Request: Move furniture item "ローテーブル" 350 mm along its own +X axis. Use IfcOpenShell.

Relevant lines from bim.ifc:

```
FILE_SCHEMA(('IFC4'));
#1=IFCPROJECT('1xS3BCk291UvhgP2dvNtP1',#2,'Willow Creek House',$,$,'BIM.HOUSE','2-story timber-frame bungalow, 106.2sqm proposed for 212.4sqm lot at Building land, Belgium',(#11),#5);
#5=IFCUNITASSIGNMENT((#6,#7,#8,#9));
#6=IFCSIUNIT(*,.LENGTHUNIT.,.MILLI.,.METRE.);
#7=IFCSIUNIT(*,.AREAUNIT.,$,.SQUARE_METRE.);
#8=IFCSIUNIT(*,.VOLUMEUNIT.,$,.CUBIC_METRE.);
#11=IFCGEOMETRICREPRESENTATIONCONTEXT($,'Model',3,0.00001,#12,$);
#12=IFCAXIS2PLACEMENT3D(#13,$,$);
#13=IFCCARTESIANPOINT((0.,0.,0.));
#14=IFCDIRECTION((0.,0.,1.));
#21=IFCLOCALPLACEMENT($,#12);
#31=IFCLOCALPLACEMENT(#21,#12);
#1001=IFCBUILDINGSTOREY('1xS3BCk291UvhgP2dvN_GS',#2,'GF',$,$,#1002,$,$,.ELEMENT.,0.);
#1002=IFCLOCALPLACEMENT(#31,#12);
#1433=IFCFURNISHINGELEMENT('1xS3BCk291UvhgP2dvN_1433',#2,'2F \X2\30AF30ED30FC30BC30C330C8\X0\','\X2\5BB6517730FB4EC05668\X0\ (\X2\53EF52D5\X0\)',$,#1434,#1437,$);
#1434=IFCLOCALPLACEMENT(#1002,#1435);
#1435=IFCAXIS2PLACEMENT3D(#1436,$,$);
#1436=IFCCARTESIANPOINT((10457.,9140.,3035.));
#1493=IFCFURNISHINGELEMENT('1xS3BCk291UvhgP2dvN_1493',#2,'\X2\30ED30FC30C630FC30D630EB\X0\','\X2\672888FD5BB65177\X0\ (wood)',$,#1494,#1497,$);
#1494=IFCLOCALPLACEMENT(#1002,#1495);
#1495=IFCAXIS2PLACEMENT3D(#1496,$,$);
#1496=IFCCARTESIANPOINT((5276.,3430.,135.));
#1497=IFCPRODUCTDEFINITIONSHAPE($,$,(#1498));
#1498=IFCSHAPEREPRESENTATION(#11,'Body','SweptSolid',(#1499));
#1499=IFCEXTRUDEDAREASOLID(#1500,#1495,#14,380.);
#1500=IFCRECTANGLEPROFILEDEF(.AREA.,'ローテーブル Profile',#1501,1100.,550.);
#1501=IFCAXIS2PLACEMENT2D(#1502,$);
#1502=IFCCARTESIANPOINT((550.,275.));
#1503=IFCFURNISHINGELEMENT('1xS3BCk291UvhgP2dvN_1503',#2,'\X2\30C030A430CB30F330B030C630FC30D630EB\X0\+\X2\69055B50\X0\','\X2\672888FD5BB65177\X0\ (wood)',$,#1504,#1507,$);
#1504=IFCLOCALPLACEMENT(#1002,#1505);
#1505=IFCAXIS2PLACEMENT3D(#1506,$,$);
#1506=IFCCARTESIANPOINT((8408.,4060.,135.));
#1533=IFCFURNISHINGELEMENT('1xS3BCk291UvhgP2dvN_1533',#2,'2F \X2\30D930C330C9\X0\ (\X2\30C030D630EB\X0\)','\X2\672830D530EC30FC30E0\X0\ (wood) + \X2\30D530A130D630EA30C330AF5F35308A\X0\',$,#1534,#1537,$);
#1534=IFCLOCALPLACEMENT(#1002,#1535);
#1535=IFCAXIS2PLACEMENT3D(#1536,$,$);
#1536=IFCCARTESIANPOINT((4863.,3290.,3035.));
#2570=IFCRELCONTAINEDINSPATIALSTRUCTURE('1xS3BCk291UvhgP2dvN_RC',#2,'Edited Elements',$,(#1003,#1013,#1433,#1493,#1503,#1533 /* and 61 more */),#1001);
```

```python
import ifcopenshell
import ifcopenshell.api.geometry
import ifcopenshell.util.placement
import ifcopenshell.util.unit

model = ifcopenshell.open("bim.ifc")
unit_scale = ifcopenshell.util.unit.calculate_unit_scale(model)

item = model.by_id(1493)
matrix = ifcopenshell.util.placement.get_local_placement(item.ObjectPlacement)
matrix[:3, 3] += matrix[:3, 0] * 0.35 / unit_scale
ifcopenshell.api.geometry.edit_object_placement(model, product=item, matrix=matrix, is_si=False)

print(ifcopenshell.util.placement.get_local_placement(item.ObjectPlacement).round(3) + 0.0)

model.write("bim-out.ifc")
```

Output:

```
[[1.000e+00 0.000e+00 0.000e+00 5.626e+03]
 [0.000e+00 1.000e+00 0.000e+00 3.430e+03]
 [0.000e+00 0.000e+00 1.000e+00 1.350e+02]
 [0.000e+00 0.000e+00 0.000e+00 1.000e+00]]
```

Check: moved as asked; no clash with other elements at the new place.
